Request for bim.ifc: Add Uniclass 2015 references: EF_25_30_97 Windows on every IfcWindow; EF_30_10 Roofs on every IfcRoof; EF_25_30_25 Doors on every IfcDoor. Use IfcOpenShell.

First a look at what the model holds.

```python
import ifcopenshell

model = ifcopenshell.open("bim.ifc")
print(model.schema)
print("classifications:", [c.Name for c in model.by_type("IfcClassification")])
for ifc_class in ("IfcDoor", "IfcRoof", "IfcStair", "IfcWall", "IfcWindow"):
    print(ifc_class, len(model.by_type(ifc_class)))
```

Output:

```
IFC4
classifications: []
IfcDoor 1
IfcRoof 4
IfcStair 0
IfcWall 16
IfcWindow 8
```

```python
import ifcopenshell
import ifcopenshell.api.classification

model = ifcopenshell.open("bim.ifc")

system = ifcopenshell.api.classification.add_classification(model, classification="Uniclass 2015")

codes = {
    "IfcWindow": ("EF_25_30_97", "Windows"),
    "IfcRoof": ("EF_30_10", "Roofs"),
    "IfcDoor": ("EF_25_30_25", "Doors"),
}
for ifc_class, (code, name) in codes.items():
    products = model.by_type(ifc_class)
    ifcopenshell.api.classification.add_reference(
        model, products=products, classification=system, identification=code, name=name
    )
    print(code, len(products))

model.write("bim_edited.ifc")
```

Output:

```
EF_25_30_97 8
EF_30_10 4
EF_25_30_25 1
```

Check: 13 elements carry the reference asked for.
